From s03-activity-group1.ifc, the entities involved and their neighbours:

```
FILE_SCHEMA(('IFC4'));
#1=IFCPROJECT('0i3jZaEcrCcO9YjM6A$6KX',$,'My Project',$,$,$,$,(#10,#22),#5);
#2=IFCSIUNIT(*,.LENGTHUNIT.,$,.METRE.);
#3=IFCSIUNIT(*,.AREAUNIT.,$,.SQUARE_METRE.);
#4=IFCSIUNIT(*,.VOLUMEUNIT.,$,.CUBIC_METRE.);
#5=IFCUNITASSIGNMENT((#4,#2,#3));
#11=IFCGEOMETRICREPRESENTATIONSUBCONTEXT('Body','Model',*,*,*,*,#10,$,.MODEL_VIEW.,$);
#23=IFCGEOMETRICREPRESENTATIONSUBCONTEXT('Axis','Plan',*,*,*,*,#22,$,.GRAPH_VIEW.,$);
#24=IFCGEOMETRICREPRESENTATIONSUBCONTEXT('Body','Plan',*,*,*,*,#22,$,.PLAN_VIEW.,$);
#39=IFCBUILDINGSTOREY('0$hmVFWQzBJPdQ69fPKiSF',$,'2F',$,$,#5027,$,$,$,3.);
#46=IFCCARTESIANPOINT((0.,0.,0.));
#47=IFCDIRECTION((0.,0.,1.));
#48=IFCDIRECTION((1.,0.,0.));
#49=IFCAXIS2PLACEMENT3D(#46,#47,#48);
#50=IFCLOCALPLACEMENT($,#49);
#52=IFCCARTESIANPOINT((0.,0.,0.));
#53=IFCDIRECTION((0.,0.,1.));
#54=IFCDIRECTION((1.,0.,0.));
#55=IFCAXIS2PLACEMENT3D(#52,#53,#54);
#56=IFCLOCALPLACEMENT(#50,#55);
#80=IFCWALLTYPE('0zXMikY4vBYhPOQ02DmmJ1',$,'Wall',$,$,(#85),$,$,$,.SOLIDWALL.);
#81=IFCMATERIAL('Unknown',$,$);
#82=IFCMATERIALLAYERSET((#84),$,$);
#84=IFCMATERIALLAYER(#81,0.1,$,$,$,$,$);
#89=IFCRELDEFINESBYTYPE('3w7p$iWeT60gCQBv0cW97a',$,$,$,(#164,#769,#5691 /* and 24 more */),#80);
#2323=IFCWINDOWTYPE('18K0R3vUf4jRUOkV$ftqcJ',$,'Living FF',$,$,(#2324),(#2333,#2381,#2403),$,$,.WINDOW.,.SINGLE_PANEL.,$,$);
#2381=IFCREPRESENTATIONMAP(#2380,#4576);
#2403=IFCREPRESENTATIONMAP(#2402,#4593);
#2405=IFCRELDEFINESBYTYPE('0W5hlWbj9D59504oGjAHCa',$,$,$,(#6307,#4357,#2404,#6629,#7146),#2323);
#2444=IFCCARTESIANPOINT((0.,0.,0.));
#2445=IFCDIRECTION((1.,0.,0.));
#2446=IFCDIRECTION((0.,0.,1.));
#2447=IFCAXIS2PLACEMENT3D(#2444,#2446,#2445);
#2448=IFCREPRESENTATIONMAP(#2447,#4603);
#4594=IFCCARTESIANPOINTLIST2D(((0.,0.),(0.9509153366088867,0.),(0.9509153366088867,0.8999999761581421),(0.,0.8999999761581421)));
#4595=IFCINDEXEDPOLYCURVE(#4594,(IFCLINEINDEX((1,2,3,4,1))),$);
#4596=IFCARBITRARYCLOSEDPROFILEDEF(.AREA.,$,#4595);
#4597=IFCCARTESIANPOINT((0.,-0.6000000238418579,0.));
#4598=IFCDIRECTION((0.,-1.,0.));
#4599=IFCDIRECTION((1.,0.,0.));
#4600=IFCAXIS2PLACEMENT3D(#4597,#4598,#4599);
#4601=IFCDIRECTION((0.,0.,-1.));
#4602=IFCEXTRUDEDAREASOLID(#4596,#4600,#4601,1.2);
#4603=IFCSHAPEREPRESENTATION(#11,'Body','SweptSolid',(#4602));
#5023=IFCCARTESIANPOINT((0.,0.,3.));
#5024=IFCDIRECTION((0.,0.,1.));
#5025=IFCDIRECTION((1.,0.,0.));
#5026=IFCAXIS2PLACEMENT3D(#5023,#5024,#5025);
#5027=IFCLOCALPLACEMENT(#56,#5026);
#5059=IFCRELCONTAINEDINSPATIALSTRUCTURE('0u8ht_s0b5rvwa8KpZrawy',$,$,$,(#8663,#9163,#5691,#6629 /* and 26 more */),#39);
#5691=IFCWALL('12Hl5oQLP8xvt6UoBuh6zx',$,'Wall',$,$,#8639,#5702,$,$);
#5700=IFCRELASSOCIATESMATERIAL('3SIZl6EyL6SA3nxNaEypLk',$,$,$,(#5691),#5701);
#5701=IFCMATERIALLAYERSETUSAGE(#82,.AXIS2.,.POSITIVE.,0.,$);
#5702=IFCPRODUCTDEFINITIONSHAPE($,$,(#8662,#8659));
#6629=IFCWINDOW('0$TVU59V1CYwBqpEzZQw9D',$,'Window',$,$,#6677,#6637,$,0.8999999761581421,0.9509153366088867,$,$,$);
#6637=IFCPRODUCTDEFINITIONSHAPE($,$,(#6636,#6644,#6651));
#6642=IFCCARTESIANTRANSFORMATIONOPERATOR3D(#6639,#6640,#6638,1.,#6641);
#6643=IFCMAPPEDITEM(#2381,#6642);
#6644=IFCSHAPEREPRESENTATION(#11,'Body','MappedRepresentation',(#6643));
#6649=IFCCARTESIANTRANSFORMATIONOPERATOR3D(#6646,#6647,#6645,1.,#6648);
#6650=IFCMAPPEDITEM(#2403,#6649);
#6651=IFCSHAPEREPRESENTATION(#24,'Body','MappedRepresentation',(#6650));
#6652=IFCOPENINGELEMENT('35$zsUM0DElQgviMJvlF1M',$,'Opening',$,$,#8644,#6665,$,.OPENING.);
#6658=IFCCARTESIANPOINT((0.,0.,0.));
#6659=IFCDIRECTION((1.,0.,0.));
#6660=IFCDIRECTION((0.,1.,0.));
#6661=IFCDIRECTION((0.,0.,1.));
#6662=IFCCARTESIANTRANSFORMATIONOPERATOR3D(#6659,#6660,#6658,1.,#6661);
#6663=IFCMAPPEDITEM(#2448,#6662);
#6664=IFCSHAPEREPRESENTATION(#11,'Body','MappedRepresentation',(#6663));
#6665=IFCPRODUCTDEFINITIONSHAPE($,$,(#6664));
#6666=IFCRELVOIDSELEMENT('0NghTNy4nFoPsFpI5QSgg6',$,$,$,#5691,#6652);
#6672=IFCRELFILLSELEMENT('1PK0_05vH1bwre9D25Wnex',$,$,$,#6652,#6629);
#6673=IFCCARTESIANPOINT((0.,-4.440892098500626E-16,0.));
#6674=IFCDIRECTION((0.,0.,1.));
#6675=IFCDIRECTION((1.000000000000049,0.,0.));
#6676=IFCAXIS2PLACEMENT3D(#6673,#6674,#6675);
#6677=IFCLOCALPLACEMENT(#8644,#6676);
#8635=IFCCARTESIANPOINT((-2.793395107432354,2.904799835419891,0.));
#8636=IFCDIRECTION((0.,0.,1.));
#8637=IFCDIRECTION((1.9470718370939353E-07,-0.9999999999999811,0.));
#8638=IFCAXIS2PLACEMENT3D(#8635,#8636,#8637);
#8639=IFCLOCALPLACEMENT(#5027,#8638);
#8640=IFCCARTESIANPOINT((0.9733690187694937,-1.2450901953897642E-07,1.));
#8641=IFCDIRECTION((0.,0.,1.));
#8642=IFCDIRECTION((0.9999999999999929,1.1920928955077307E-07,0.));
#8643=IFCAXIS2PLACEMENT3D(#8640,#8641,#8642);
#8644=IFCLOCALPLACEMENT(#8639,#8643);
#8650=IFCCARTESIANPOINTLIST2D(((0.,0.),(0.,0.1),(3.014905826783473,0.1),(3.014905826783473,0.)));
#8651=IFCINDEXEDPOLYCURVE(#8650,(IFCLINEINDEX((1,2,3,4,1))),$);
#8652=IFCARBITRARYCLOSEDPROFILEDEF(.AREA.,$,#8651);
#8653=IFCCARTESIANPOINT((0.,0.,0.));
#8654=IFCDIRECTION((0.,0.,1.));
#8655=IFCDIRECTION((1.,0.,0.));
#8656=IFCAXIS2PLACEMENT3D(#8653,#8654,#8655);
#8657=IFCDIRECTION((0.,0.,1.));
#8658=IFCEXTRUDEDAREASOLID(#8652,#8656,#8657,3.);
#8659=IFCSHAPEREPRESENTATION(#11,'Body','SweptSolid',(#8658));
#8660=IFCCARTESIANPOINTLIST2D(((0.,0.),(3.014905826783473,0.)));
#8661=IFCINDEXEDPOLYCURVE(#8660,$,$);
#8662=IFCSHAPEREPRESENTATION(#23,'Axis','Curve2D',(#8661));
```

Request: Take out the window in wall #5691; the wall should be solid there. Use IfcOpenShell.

```python
import ifcopenshell
import ifcopenshell.api.feature
import ifcopenshell.api.root
import ifcopenshell.geom
import ifcopenshell.util.shape

model = ifcopenshell.open("s03-activity-group1.ifc")
settings = ifcopenshell.geom.settings()


def volume(element):
    """Net volume in cubic metres, openings subtracted."""
    shape = ifcopenshell.geom.create_shape(settings, element)
    return ifcopenshell.util.shape.get_volume(shape.geometry)


window = model.by_guid("0$TVU59V1CYwBqpEzZQw9D")
opening = window.FillsVoids[0].RelatingOpeningElement
wall = opening.VoidsElements[0].RelatingBuildingElement
before = volume(wall)

ifcopenshell.api.root.remove_product(model, product=window)
ifcopenshell.api.feature.remove_feature(model, feature=opening)

after = volume(wall)

print(f"wall volume {before:.3f} -> {after:.3f} m3")

model.write("s03-activity-group1_edited.ifc")
```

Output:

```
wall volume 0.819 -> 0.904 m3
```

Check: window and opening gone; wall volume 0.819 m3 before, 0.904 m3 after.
